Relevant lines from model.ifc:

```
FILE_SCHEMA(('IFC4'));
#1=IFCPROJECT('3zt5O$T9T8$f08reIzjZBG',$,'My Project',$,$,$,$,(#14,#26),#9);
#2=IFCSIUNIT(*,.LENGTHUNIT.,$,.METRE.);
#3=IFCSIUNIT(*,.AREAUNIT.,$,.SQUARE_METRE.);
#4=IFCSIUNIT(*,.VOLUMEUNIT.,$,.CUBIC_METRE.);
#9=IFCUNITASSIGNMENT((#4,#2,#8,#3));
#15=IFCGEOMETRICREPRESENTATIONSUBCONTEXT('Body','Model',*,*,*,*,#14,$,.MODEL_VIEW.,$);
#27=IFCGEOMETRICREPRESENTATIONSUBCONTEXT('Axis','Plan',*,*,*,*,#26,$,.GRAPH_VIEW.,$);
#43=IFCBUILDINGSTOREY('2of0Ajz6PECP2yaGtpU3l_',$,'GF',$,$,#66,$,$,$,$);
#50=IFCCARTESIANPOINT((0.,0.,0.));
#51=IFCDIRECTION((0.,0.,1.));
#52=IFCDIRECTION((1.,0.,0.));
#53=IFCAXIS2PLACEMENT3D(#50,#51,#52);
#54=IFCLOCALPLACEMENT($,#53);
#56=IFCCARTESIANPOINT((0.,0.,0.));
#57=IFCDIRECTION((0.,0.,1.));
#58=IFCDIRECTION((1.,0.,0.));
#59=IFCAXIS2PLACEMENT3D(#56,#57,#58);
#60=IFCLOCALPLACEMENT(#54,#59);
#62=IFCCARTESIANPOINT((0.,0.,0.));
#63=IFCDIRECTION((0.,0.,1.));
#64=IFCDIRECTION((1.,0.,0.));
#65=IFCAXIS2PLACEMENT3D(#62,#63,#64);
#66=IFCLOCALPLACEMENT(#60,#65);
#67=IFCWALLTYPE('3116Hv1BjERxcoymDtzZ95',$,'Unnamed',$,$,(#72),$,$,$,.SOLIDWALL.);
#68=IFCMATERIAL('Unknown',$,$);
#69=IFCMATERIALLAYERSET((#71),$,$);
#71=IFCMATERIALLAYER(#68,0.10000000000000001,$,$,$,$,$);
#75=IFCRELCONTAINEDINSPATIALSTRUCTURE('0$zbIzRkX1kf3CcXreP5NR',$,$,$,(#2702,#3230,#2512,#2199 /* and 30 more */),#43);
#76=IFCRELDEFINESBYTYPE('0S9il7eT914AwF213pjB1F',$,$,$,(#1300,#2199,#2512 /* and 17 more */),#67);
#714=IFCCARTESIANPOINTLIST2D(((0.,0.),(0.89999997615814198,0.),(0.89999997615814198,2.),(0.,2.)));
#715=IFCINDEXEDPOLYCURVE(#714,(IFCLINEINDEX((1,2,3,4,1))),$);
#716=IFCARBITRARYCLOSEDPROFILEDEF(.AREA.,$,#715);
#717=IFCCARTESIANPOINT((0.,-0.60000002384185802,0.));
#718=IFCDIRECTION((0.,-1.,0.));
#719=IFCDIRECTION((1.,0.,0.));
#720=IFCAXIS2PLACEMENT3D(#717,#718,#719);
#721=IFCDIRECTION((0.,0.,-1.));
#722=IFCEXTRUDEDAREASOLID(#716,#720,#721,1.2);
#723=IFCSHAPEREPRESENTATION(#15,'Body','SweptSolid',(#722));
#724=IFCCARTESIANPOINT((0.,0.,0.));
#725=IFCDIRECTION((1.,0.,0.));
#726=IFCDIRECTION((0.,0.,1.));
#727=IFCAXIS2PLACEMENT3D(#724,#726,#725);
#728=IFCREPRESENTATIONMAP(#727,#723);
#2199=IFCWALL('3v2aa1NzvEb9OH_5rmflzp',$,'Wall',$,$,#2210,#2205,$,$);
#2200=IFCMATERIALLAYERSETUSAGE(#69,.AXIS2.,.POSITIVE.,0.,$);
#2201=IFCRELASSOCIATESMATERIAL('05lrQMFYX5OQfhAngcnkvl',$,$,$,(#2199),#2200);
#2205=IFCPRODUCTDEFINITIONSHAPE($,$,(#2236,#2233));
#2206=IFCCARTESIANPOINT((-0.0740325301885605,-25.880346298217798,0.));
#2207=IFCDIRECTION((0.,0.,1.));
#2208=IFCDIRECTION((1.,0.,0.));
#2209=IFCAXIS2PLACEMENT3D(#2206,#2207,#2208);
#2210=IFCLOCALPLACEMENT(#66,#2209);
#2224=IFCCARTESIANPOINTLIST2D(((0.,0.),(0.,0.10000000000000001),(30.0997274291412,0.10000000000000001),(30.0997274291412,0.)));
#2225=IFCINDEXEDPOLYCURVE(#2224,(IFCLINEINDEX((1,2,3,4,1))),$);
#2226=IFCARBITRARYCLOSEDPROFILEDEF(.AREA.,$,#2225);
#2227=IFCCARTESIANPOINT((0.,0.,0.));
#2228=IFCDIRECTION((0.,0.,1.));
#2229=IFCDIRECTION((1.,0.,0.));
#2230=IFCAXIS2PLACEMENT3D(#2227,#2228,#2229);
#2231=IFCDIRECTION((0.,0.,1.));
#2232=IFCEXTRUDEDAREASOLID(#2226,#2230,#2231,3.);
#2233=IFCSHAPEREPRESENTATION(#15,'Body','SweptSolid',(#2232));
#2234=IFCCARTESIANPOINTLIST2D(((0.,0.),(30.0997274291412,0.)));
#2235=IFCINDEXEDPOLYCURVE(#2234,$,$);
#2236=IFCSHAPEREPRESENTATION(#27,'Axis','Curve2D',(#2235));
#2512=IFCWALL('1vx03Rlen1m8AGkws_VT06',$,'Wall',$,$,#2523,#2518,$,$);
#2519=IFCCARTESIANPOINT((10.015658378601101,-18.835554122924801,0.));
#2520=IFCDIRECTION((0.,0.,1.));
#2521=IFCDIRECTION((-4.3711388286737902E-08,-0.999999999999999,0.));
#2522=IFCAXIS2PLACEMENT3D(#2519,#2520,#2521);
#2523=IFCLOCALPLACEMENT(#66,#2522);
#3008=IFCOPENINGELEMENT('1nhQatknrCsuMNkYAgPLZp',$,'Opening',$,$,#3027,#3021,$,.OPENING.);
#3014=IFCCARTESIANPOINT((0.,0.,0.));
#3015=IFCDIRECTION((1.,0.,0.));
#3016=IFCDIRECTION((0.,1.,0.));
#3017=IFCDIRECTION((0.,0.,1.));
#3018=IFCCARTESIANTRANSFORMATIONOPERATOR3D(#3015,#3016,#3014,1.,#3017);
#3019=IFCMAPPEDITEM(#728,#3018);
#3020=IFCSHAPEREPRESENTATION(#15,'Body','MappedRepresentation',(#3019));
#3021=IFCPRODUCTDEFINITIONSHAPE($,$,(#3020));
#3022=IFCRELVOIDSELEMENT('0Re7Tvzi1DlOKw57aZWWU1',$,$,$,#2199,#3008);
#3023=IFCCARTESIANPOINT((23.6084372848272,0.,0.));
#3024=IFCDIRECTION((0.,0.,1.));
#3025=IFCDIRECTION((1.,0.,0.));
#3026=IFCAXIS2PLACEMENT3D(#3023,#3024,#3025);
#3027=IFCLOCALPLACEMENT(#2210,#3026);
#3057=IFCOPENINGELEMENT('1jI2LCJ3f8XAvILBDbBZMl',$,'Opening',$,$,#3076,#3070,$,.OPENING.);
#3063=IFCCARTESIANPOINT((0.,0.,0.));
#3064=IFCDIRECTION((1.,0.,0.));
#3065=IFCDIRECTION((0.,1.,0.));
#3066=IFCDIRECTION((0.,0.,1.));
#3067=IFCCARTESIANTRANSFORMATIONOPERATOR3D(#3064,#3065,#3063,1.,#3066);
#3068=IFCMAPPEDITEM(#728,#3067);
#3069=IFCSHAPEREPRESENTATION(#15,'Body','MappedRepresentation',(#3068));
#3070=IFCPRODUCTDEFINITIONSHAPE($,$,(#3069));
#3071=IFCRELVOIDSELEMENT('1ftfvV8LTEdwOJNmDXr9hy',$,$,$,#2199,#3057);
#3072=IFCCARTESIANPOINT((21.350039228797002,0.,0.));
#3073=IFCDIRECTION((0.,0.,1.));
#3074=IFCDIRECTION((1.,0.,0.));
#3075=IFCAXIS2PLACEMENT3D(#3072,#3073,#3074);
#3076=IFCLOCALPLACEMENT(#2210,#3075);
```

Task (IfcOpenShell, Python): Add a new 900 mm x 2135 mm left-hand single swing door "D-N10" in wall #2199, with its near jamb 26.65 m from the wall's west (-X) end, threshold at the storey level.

```python
import numpy as np
import ifcopenshell
import ifcopenshell.api.feature
import ifcopenshell.api.geometry
import ifcopenshell.api.root
import ifcopenshell.api.spatial
import ifcopenshell.geom
import ifcopenshell.util.element
import ifcopenshell.util.placement
import ifcopenshell.util.representation
import ifcopenshell.util.shape
import ifcopenshell.util.unit

model = ifcopenshell.open("model.ifc")
unit_scale = ifcopenshell.util.unit.calculate_unit_scale(model)
settings = ifcopenshell.geom.settings()


def volume(element):
    """Net volume in cubic metres, openings subtracted."""
    shape = ifcopenshell.geom.create_shape(settings, element)
    return ifcopenshell.util.shape.get_volume(shape.geometry)


wall = model.by_guid("3v2aa1NzvEb9OH_5rmflzp")
storey = ifcopenshell.util.element.get_container(wall, ifc_class="IfcBuildingStorey")
context = ifcopenshell.util.representation.get_context(model, "Model", "Body", "MODEL_VIEW")
before = volume(wall)

width, height, from_end, sill = 0.9, 2.135, 26.65, 0.0  # metres

# The wall runs along its own X axis, and the end named is its -X end.
wall_shape = ifcopenshell.geom.create_shape(settings, wall)
x, y, z = ifcopenshell.util.shape.get_vertices(wall_shape.geometry).T
start = x.min() + from_end
face, thickness = float(y.min()), float(y.max() - y.min())
wall_matrix = ifcopenshell.util.placement.get_local_placement(wall.ObjectPlacement)
level = ifcopenshell.util.placement.get_local_placement(storey.ObjectPlacement)[2, 3]


def in_wall(x, y):
    """Placement at x, y metres in the wall's axes, at sill height."""
    matrix = wall_matrix.copy()
    matrix[:, 3] = wall_matrix @ np.array([x / unit_scale, y / unit_scale, 0.0, 1.0])
    matrix[2, 3] = level + sill / unit_scale
    return matrix


# Opening: a box that overshoots both wall faces by 50 mm.
opening = ifcopenshell.api.root.create_entity(model, ifc_class="IfcOpeningElement", predefined_type="OPENING")
box = ifcopenshell.api.geometry.add_wall_representation(
    model, context=context, length=width, height=height, thickness=thickness + 0.1
)
ifcopenshell.api.geometry.assign_representation(model, product=opening, representation=box)
ifcopenshell.api.geometry.edit_object_placement(model, product=opening, matrix=in_wall(start, face - 0.05), is_si=False)
ifcopenshell.api.feature.add_feature(model, feature=opening, element=wall)

door = ifcopenshell.api.root.create_entity(model, ifc_class="IfcDoor", name="D-N10", predefined_type="DOOR")
door.OverallWidth, door.OverallHeight = width / unit_scale, height / unit_scale
door.OperationType = "SINGLE_SWING_LEFT"
body = ifcopenshell.api.geometry.add_door_representation(
    model,
    context=context,
    overall_width=door.OverallWidth,
    overall_height=door.OverallHeight,
    operation_type="SINGLE_SWING_LEFT",
    lining_properties={"LiningDepth": thickness / unit_scale, "ThresholdDepth": thickness / unit_scale},
)
ifcopenshell.api.geometry.assign_representation(model, product=door, representation=body)
ifcopenshell.api.spatial.assign_container(model, products=[door], relating_structure=storey)
ifcopenshell.api.feature.add_filling(model, opening=opening, element=door)

# The lining spans the wall, so the door starts at the wall face.
ifcopenshell.api.geometry.edit_object_placement(model, product=door, matrix=in_wall(start, face), is_si=False)

after = volume(wall)

print(f"wall volume {before:.3f} -> {after:.3f} m3")

model.write("model_v2.ifc")
```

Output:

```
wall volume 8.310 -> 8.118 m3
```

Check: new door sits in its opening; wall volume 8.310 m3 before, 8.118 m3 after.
